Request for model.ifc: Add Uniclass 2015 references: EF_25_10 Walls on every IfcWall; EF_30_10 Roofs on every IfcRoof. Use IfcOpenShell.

First a look at what the model holds.

```python
import ifcopenshell

model = ifcopenshell.open("model.ifc")
print(model.schema)
print("classifications:", [c.Name for c in model.by_type("IfcClassification")])
for ifc_class in ("IfcDoor", "IfcRoof", "IfcStair", "IfcWall", "IfcWindow"):
    print(ifc_class, len(model.by_type(ifc_class)))
```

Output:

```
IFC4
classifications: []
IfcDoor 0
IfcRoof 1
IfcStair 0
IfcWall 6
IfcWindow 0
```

```python
import ifcopenshell
import ifcopenshell.api.classification

model = ifcopenshell.open("model.ifc")

system = ifcopenshell.api.classification.add_classification(model, classification="Uniclass 2015")

codes = {
    "IfcWall": ("EF_25_10", "Walls"),
    "IfcRoof": ("EF_30_10", "Roofs"),
}
for ifc_class, (code, name) in codes.items():
    products = model.by_type(ifc_class)
    ifcopenshell.api.classification.add_reference(
        model, products=products, classification=system, identification=code, name=name
    )
    print(code, len(products))

model.write("model-out.ifc")
```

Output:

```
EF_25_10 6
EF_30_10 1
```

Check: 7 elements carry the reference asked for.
